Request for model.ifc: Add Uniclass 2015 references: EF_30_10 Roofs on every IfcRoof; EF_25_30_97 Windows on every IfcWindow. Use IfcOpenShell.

First a look at what the model holds.

```python
import ifcopenshell

model = ifcopenshell.open("model.ifc")
print(model.schema)
print("classifications:", [c.Name for c in model.by_type("IfcClassification")])
for ifc_class in ("IfcDoor", "IfcRoof", "IfcStair", "IfcWall", "IfcWindow"):
    print(ifc_class, len(model.by_type(ifc_class)))
```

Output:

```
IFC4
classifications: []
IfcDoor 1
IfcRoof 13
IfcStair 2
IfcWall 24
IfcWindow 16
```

```python
import ifcopenshell
import ifcopenshell.api.classification

model = ifcopenshell.open("model.ifc")

system = ifcopenshell.api.classification.add_classification(model, classification="Uniclass 2015")

codes = {
    "IfcRoof": ("EF_30_10", "Roofs"),
    "IfcWindow": ("EF_25_30_97", "Windows"),
}
for ifc_class, (code, name) in codes.items():
    products = model.by_type(ifc_class)
    ifcopenshell.api.classification.add_reference(
        model, products=products, classification=system, identification=code, name=name
    )
    print(code, len(products))

model.write("model_updated.ifc")
```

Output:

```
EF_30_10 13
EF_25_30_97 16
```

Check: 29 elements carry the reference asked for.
